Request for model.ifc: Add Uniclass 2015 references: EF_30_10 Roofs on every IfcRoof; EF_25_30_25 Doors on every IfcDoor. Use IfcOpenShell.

First a look at what the model holds.

```python
import ifcopenshell

model = ifcopenshell.open("model.ifc")
print(model.schema)
print("classifications:", [c.Name for c in model.by_type("IfcClassification")])
for ifc_class in ("IfcDoor", "IfcRoof", "IfcStair", "IfcWall", "IfcWindow"):
    print(ifc_class, len(model.by_type(ifc_class)))
```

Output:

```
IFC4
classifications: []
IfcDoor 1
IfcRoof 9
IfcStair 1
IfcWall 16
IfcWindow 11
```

```python
import ifcopenshell
import ifcopenshell.api.classification

model = ifcopenshell.open("model.ifc")

system = ifcopenshell.api.classification.add_classification(model, classification="Uniclass 2015")

codes = {
    "IfcRoof": ("EF_30_10", "Roofs"),
    "IfcDoor": ("EF_25_30_25", "Doors"),
}
for ifc_class, (code, name) in codes.items():
    products = model.by_type(ifc_class)
    ifcopenshell.api.classification.add_reference(
        model, products=products, classification=system, identification=code, name=name
    )
    print(code, len(products))

model.write("model_updated.ifc")
```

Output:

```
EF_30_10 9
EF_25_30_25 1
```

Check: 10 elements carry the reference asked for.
